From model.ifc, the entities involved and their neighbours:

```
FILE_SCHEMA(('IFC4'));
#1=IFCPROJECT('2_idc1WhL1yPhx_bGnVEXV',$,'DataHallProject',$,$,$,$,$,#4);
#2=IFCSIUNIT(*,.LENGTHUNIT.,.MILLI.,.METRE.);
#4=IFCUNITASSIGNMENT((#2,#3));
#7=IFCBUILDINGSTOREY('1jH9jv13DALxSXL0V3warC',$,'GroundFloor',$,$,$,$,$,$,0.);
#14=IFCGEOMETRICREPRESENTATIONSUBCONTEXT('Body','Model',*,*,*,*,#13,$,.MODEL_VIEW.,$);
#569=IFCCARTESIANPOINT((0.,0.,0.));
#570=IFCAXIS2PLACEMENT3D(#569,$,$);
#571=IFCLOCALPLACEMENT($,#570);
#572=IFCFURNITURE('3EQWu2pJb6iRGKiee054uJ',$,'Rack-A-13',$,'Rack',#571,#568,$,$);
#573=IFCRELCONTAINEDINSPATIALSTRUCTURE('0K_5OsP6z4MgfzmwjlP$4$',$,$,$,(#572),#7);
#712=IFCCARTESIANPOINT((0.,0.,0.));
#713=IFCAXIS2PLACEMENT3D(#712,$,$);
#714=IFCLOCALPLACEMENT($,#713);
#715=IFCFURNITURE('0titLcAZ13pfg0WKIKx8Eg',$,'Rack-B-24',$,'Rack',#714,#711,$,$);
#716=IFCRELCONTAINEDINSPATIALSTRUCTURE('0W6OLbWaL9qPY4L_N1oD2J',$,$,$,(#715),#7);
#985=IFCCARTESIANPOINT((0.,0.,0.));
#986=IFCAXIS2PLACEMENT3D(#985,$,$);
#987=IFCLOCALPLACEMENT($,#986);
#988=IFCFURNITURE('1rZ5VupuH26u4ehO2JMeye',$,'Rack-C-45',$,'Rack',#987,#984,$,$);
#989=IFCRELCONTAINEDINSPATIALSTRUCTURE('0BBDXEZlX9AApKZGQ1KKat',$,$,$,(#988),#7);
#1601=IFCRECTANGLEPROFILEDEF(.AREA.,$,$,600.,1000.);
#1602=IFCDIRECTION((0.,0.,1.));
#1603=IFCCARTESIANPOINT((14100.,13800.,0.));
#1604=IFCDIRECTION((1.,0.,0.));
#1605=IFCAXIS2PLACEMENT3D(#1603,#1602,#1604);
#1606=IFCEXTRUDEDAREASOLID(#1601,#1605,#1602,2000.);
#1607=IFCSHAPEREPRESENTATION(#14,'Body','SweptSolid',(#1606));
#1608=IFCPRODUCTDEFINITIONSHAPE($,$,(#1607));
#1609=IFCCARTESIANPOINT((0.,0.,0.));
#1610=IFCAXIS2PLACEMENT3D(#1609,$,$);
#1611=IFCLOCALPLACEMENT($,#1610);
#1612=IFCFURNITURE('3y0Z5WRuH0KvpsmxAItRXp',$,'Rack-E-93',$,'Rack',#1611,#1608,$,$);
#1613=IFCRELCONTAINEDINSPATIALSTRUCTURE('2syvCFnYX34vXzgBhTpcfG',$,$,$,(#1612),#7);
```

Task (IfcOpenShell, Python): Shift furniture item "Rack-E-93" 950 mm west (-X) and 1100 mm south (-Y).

```python
import ifcopenshell
import ifcopenshell.api.geometry
import ifcopenshell.util.placement
import ifcopenshell.util.unit

model = ifcopenshell.open("model.ifc")
unit_scale = ifcopenshell.util.unit.calculate_unit_scale(model)

item = model.by_guid("3y0Z5WRuH0KvpsmxAItRXp")
matrix = ifcopenshell.util.placement.get_local_placement(item.ObjectPlacement)
matrix[0, 3] -= 0.95 / unit_scale
matrix[1, 3] -= 1.1 / unit_scale
ifcopenshell.api.geometry.edit_object_placement(model, product=item, matrix=matrix, is_si=False)

print(ifcopenshell.util.placement.get_local_placement(item.ObjectPlacement).round(3) + 0.0)

model.write("model_v2.ifc")
```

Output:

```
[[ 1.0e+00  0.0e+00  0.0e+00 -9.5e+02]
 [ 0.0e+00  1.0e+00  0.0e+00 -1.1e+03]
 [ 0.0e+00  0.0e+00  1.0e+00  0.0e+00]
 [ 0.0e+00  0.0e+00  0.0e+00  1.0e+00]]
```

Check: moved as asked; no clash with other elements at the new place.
